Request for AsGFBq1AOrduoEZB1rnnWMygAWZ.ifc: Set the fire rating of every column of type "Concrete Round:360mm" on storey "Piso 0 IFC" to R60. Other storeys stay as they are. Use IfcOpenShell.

First a look at what the model holds.

```python
import ifcopenshell
import ifcopenshell.util.element

model = ifcopenshell.open("AsGFBq1AOrduoEZB1rnnWMygAWZ.ifc")
print(model.schema)
storey = next(s for s in model.by_type("IfcBuildingStorey") if s.Name == "Piso 0 IFC")
columns = [e for e in ifcopenshell.util.element.get_decomposition(storey) if e.is_a("IfcColumn")]
seen = {}
for e in columns:
    element_type = ifcopenshell.util.element.get_type(e)
    key = (element_type.Name if element_type != e and element_type else None, ifcopenshell.util.element.get_pset(e, "Pset_ColumnCommon", "FireRating"))
    seen[key] = seen.get(key, 0) + 1
for (name, value), count in sorted(seen.items(), key=str):
    print(count, "x", name, "|", value)
```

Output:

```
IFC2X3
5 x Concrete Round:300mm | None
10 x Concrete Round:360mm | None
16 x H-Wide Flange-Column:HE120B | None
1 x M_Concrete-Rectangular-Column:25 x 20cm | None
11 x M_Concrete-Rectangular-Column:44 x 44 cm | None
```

```python
import ifcopenshell
import ifcopenshell.api.pset
import ifcopenshell.util.element

model = ifcopenshell.open("AsGFBq1AOrduoEZB1rnnWMygAWZ.ifc")

storey = next(s for s in model.by_type("IfcBuildingStorey") if s.Name == "Piso 0 IFC")
columns = [e for e in ifcopenshell.util.element.get_decomposition(storey) if e.is_a("IfcColumn")]

count = 0
for e in columns:
    element_type = ifcopenshell.util.element.get_type(e)
    if element_type in (None, e) or element_type.Name != "Concrete Round:360mm":
        continue
    # add_pset returns the element's existing set when there is one.
    pset = ifcopenshell.api.pset.add_pset(model, product=e, name="Pset_ColumnCommon")
    ifcopenshell.api.pset.edit_pset(model, pset=pset, properties={"FireRating": "R60"})
    count += 1

print(count, "columns updated")

model.write("AsGFBq1AOrduoEZB1rnnWMygAWZ-out.ifc")
```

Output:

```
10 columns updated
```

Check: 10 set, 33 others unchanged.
